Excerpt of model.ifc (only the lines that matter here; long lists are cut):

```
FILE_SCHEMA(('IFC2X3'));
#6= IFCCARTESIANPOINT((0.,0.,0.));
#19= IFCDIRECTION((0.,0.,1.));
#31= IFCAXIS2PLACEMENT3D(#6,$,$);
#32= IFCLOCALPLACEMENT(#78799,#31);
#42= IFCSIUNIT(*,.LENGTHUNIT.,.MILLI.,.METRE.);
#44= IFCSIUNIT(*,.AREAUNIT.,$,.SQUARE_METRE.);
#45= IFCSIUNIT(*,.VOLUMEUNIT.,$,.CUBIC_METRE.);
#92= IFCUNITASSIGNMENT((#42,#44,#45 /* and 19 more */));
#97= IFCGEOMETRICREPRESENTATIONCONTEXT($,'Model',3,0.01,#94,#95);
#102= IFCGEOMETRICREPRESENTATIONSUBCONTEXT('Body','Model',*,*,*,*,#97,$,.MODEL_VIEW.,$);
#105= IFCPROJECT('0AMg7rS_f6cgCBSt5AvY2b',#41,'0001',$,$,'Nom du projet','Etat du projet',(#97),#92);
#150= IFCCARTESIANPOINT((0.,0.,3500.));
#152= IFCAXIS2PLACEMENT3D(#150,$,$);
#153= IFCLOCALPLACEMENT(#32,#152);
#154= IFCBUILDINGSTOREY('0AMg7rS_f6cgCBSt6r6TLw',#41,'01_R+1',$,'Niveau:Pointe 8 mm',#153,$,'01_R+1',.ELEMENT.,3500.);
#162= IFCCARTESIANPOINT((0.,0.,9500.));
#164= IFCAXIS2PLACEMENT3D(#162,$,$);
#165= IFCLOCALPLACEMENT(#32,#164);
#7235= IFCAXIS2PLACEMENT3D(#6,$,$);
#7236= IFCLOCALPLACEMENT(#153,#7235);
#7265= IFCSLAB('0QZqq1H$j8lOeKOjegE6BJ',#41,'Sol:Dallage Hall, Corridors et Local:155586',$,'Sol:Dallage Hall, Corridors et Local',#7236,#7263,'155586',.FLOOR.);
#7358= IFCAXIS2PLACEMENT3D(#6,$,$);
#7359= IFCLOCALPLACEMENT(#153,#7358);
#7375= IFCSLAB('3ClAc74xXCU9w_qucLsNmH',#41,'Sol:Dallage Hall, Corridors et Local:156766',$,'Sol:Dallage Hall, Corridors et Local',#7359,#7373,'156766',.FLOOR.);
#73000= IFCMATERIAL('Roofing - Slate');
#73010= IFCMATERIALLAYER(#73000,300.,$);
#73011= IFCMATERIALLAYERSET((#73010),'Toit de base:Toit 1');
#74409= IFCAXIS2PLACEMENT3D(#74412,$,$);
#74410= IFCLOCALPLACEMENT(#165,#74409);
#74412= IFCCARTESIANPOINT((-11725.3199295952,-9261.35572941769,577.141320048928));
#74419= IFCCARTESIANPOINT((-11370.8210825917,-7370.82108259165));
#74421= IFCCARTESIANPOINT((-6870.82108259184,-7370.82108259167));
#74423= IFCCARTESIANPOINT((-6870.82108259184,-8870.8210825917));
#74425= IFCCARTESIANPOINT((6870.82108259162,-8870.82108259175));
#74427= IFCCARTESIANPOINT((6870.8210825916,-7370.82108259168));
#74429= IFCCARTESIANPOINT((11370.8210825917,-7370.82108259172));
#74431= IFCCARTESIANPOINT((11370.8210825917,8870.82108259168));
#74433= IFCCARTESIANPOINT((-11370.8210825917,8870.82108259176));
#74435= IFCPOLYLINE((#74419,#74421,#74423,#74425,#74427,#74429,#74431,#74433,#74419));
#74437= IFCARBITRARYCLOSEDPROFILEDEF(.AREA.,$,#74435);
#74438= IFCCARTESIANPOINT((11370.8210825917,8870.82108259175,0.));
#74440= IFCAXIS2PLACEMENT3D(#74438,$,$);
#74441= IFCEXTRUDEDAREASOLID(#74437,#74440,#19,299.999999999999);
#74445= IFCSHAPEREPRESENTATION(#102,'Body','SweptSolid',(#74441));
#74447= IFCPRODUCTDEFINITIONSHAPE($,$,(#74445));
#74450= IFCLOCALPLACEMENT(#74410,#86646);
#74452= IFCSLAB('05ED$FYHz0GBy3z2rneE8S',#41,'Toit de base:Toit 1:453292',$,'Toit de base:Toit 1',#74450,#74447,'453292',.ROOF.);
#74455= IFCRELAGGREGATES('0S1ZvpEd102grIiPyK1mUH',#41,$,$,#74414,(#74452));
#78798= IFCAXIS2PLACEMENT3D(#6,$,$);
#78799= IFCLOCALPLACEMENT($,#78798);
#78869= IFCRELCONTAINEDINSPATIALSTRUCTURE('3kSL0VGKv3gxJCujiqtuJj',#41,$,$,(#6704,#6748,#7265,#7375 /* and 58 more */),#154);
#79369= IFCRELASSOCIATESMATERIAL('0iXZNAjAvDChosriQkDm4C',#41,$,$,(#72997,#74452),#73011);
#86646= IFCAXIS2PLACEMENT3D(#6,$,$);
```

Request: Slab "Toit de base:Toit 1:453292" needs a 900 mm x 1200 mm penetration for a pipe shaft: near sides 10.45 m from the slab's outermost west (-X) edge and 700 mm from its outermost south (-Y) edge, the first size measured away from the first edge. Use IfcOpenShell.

```python
import numpy as np
import ifcopenshell
import ifcopenshell.api.feature
import ifcopenshell.api.geometry
import ifcopenshell.api.root
import ifcopenshell.geom
import ifcopenshell.util.placement
import ifcopenshell.util.representation
import ifcopenshell.util.shape
import ifcopenshell.util.unit

model = ifcopenshell.open("model.ifc")
unit_scale = ifcopenshell.util.unit.calculate_unit_scale(model)
settings = ifcopenshell.geom.settings()


def volume(element):
    """Net volume in cubic metres, openings subtracted."""
    shape = ifcopenshell.geom.create_shape(settings, element)
    return ifcopenshell.util.shape.get_volume(shape.geometry)


slab = model.by_guid("05ED$FYHz0GBy3z2rneE8S")
before = volume(slab)

# Extent in the slab's own axes, in metres. The edges named are its -X and -Y sides.
slab_shape = ifcopenshell.geom.create_shape(settings, slab)
vertices = ifcopenshell.util.shape.get_vertices(slab_shape.geometry)
x_min, y_min, bottom = vertices.min(axis=0)
top = vertices[:, 2].max()

opening = ifcopenshell.api.root.create_entity(model, ifc_class="IfcOpeningElement", name="Pipe shaft opening")
context = ifcopenshell.util.representation.get_context(model, "Model", "Body", "MODEL_VIEW")
width, depth = 0.9, 1.2
outline = [(0.0, 0.0), (width, 0.0), (width, depth), (0.0, depth), (0.0, 0.0)]
# Overshoot both faces by 50 mm so the cut is clean.
shape = ifcopenshell.api.geometry.add_slab_representation(
    model, context=context, depth=top - bottom + 0.1, polyline=outline
)
ifcopenshell.api.geometry.assign_representation(model, product=opening, representation=shape)

matrix = ifcopenshell.util.placement.get_local_placement(slab.ObjectPlacement)
matrix[:, 3] = matrix @ np.append(np.array([x_min + 10.45, y_min + 0.7, bottom - 0.05]) / unit_scale, 1.0)
ifcopenshell.api.geometry.edit_object_placement(model, product=opening, matrix=matrix, is_si=False)
ifcopenshell.api.feature.add_feature(model, feature=opening, element=slab)

after = volume(slab)

print(f"slab volume {before:.3f} -> {after:.3f} m3")

model.write("model_rev.ifc")
```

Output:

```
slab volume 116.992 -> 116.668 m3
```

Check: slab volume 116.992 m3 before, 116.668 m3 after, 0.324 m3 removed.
